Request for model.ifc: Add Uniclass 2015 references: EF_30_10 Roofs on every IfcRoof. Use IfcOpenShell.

First a look at what the model holds.

```python
import ifcopenshell

model = ifcopenshell.open("model.ifc")
print(model.schema)
print("classifications:", [c.Name for c in model.by_type("IfcClassification")])
for ifc_class in ("IfcDoor", "IfcRoof", "IfcStair", "IfcWall", "IfcWindow"):
    print(ifc_class, len(model.by_type(ifc_class)))
```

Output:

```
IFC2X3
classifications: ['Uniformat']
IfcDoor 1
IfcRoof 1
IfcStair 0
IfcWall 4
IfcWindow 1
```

```python
import ifcopenshell
import ifcopenshell.api.classification

model = ifcopenshell.open("model.ifc")

# IFC2X3 requires Source and Edition and has no link from the project to the system.
system = model.create_entity("IfcClassification", Source="NBS", Edition="2015", Name="Uniclass 2015")

codes = {
    "IfcRoof": ("EF_30_10", "Roofs"),
}
for ifc_class, (code, name) in codes.items():
    products = model.by_type(ifc_class)
    ifcopenshell.api.classification.add_reference(
        model, products=products, classification=system, identification=code, name=name
    )
    print(code, len(products))

model.write("model_edited.ifc")
```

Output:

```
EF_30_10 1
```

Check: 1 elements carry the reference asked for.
